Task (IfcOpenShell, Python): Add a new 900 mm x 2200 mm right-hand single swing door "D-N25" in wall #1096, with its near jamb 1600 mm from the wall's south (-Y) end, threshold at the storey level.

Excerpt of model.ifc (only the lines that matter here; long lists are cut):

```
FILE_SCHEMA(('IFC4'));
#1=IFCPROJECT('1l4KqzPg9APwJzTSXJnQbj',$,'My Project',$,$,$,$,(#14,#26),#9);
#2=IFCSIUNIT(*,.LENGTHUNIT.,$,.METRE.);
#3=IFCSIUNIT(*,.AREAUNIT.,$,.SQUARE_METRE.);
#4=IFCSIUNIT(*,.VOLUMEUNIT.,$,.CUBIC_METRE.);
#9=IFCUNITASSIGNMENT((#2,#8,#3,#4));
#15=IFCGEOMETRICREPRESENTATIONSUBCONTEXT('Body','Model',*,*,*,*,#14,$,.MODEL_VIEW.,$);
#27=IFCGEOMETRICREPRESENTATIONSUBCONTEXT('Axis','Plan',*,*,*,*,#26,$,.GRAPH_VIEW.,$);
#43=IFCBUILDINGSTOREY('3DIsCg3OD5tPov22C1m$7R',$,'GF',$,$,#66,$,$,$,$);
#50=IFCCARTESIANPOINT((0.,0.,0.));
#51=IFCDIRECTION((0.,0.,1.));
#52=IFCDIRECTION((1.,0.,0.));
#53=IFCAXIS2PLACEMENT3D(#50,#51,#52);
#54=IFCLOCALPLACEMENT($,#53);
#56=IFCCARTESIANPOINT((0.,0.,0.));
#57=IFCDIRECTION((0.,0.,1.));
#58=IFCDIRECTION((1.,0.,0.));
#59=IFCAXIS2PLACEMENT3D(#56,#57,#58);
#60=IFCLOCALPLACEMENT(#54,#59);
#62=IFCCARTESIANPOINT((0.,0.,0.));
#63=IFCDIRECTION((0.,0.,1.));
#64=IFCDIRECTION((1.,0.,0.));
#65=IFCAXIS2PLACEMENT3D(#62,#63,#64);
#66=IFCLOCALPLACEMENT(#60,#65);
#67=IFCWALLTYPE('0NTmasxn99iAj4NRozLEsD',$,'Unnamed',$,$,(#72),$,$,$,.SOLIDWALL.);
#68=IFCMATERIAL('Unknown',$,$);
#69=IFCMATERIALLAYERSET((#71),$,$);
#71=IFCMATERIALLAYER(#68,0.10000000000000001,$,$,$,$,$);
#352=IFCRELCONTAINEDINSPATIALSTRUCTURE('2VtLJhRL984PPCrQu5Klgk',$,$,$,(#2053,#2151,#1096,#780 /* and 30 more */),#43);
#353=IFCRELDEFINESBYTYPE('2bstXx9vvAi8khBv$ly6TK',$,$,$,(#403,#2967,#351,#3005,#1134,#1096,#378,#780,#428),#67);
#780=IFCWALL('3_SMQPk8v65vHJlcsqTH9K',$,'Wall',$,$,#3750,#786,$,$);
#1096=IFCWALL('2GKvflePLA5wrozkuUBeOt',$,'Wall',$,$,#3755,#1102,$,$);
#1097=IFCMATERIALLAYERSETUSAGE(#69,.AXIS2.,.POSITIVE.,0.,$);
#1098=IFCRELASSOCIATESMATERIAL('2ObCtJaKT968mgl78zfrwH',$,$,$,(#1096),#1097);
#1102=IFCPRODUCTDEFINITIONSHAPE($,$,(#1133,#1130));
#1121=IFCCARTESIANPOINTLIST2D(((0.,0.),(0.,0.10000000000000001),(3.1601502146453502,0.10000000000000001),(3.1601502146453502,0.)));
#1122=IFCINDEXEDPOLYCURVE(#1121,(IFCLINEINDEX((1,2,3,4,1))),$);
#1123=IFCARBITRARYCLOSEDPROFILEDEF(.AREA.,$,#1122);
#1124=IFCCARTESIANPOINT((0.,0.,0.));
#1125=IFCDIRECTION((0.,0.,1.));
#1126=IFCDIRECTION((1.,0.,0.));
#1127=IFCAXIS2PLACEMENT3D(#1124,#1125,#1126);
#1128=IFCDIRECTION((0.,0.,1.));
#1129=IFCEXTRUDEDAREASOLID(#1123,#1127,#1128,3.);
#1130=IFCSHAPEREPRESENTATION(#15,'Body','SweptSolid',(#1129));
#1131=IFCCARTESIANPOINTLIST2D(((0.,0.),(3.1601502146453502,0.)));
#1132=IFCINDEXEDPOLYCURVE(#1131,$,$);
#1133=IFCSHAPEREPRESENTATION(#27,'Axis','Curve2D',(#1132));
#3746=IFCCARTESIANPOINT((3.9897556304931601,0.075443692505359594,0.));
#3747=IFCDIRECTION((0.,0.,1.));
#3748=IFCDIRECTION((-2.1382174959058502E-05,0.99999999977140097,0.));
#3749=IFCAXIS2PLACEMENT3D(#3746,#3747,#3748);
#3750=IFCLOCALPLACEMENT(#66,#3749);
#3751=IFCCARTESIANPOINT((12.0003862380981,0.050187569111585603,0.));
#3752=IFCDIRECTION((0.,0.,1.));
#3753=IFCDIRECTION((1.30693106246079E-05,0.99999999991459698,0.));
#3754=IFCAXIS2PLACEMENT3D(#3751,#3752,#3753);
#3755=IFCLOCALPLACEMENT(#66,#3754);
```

```python
import numpy as np
import ifcopenshell
import ifcopenshell.api.feature
import ifcopenshell.api.geometry
import ifcopenshell.api.root
import ifcopenshell.api.spatial
import ifcopenshell.geom
import ifcopenshell.util.element
import ifcopenshell.util.placement
import ifcopenshell.util.representation
import ifcopenshell.util.shape
import ifcopenshell.util.unit

model = ifcopenshell.open("model.ifc")
unit_scale = ifcopenshell.util.unit.calculate_unit_scale(model)
settings = ifcopenshell.geom.settings()


def volume(element):
    """Net volume in cubic metres, openings subtracted."""
    shape = ifcopenshell.geom.create_shape(settings, element)
    return ifcopenshell.util.shape.get_volume(shape.geometry)


wall = model.by_guid("2GKvflePLA5wrozkuUBeOt")
storey = ifcopenshell.util.element.get_container(wall, ifc_class="IfcBuildingStorey")
context = ifcopenshell.util.representation.get_context(model, "Model", "Body", "MODEL_VIEW")
before = volume(wall)

width, height, from_end, sill = 0.9, 2.2, 1.6, 0.0  # metres

# The wall runs along its own X axis, and the end named is its -X end.
wall_shape = ifcopenshell.geom.create_shape(settings, wall)
x, y, z = ifcopenshell.util.shape.get_vertices(wall_shape.geometry).T
start = x.min() + from_end
face, thickness = float(y.min()), float(y.max() - y.min())
wall_matrix = ifcopenshell.util.placement.get_local_placement(wall.ObjectPlacement)
level = ifcopenshell.util.placement.get_local_placement(storey.ObjectPlacement)[2, 3]


def in_wall(x, y):
    """Placement at x, y metres in the wall's axes, at sill height."""
    matrix = wall_matrix.copy()
    matrix[:, 3] = wall_matrix @ np.array([x / unit_scale, y / unit_scale, 0.0, 1.0])
    matrix[2, 3] = level + sill / unit_scale
    return matrix


# Opening: a box that overshoots both wall faces by 50 mm.
opening = ifcopenshell.api.root.create_entity(model, ifc_class="IfcOpeningElement", predefined_type="OPENING")
box = ifcopenshell.api.geometry.add_wall_representation(
    model, context=context, length=width, height=height, thickness=thickness + 0.1
)
ifcopenshell.api.geometry.assign_representation(model, product=opening, representation=box)
ifcopenshell.api.geometry.edit_object_placement(model, product=opening, matrix=in_wall(start, face - 0.05), is_si=False)
ifcopenshell.api.feature.add_feature(model, feature=opening, element=wall)

door = ifcopenshell.api.root.create_entity(model, ifc_class="IfcDoor", name="D-N25", predefined_type="DOOR")
door.OverallWidth, door.OverallHeight = width / unit_scale, height / unit_scale
door.OperationType = "SINGLE_SWING_RIGHT"
body = ifcopenshell.api.geometry.add_door_representation(
    model,
    context=context,
    overall_width=door.OverallWidth,
    overall_height=door.OverallHeight,
    operation_type="SINGLE_SWING_RIGHT",
    lining_properties={"LiningDepth": thickness / unit_scale, "ThresholdDepth": thickness / unit_scale},
)
ifcopenshell.api.geometry.assign_representation(model, product=door, representation=body)
ifcopenshell.api.spatial.assign_container(model, products=[door], relating_structure=storey)
ifcopenshell.api.feature.add_filling(model, opening=opening, element=door)

# The lining spans the wall, so the door starts at the wall face.
ifcopenshell.api.geometry.edit_object_placement(model, product=door, matrix=in_wall(start, face), is_si=False)

after = volume(wall)

print(f"wall volume {before:.3f} -> {after:.3f} m3")

model.write("model_edited.ifc")
```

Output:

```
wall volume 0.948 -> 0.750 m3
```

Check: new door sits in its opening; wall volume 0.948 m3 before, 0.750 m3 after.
